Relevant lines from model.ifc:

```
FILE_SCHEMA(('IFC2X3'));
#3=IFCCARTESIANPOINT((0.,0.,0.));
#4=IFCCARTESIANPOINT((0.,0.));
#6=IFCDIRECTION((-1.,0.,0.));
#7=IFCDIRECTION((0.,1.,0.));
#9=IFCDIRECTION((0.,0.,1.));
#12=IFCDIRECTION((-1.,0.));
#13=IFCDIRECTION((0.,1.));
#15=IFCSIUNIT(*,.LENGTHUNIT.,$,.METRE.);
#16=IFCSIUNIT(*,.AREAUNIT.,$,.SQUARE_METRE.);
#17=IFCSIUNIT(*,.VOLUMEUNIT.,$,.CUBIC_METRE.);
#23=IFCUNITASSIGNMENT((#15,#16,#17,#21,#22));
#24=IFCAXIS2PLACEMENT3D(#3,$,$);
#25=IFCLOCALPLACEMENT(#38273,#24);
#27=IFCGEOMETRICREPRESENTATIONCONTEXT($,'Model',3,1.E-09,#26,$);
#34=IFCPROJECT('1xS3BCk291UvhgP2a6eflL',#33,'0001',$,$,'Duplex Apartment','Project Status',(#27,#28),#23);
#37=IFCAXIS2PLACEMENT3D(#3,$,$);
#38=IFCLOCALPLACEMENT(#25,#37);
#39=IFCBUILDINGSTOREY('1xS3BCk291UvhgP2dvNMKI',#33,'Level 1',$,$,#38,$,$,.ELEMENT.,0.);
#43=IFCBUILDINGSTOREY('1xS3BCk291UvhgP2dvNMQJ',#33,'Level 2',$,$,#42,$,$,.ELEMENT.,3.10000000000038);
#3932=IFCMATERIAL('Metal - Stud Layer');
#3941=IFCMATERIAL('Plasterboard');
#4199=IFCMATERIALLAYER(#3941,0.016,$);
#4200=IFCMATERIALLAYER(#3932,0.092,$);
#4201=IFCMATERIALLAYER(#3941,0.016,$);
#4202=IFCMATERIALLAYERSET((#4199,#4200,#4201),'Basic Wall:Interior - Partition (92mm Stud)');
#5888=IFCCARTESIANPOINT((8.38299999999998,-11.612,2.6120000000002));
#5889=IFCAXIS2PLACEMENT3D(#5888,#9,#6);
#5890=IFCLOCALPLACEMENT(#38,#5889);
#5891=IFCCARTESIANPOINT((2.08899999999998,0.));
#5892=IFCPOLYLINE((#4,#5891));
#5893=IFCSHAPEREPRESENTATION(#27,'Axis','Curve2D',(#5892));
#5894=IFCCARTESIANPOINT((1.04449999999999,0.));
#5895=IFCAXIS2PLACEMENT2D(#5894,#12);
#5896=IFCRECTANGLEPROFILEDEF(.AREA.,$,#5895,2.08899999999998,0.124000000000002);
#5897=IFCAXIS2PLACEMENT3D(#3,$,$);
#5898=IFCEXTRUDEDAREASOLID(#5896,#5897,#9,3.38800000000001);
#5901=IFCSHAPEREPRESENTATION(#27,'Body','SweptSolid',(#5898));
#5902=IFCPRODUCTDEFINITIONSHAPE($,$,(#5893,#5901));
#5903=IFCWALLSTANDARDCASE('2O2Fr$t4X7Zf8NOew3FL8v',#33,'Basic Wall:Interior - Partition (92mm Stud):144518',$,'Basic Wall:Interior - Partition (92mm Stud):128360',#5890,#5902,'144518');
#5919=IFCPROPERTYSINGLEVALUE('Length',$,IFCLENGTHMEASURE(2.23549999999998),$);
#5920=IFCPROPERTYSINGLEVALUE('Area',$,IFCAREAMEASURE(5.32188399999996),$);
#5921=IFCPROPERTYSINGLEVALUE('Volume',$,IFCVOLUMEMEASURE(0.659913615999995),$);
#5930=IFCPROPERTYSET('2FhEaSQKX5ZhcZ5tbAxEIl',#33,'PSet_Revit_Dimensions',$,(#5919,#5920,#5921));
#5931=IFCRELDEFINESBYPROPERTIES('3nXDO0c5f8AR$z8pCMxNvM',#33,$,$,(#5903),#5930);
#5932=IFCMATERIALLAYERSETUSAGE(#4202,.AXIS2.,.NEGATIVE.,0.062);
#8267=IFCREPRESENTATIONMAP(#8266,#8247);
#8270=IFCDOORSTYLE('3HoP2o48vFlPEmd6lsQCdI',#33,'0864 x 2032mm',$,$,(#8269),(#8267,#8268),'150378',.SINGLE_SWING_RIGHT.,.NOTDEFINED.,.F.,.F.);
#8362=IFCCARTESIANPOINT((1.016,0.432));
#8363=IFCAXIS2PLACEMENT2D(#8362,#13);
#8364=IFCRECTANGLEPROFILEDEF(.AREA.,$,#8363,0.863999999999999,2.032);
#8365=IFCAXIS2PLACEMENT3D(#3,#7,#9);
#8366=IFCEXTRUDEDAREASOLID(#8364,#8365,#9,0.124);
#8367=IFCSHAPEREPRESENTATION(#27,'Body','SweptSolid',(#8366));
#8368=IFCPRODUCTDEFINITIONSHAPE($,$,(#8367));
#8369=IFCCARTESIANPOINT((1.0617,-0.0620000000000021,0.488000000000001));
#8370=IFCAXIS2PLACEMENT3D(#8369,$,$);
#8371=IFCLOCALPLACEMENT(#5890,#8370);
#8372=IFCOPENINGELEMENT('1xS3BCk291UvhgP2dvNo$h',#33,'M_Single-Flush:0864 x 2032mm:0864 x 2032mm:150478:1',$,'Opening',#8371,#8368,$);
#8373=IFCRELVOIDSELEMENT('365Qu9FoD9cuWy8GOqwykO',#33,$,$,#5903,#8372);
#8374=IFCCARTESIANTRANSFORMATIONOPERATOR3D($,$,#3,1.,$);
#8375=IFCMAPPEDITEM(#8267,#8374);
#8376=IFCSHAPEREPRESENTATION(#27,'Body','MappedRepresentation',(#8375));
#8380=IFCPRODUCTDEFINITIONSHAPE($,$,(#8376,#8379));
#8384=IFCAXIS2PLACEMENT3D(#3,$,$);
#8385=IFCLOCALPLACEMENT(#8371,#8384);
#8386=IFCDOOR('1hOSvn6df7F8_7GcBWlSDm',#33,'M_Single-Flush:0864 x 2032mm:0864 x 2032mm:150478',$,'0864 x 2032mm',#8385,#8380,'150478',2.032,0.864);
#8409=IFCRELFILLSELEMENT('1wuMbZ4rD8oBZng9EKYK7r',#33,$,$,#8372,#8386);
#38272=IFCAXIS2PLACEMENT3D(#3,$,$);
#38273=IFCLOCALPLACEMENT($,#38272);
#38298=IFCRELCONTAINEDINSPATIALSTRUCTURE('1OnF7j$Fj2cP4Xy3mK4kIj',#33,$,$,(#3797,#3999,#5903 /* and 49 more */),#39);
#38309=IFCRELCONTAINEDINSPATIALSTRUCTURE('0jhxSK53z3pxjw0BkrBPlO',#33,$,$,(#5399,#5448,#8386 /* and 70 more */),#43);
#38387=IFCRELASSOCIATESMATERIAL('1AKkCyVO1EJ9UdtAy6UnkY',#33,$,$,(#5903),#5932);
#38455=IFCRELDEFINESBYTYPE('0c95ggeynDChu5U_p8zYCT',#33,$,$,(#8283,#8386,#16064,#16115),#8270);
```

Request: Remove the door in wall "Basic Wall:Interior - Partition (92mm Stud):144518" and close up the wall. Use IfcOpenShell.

```python
import ifcopenshell
import ifcopenshell.api.feature
import ifcopenshell.api.pset
import ifcopenshell.api.root
import ifcopenshell.geom
import ifcopenshell.util.element
import ifcopenshell.util.shape
import ifcopenshell.util.unit

model = ifcopenshell.open("model.ifc")
area_scale = ifcopenshell.util.unit.calculate_unit_scale(model, "AREAUNIT")
volume_scale = ifcopenshell.util.unit.calculate_unit_scale(model, "VOLUMEUNIT")
settings = ifcopenshell.geom.settings()


def volume(element):
    """Net volume in cubic metres, openings subtracted."""
    shape = ifcopenshell.geom.create_shape(settings, element)
    return ifcopenshell.util.shape.get_volume(shape.geometry)


door = model.by_guid("1hOSvn6df7F8_7GcBWlSDm")
opening = door.FillsVoids[0].RelatingOpeningElement
wall = opening.VoidsElements[0].RelatingBuildingElement
before = volume(wall)

ifcopenshell.api.root.remove_product(model, product=door)
ifcopenshell.api.feature.remove_feature(model, feature=opening)

after = volume(wall)
thickness = 0.124  # wall thickness in metres

# Update the wall's stored quantities.
pset = model.by_id(ifcopenshell.util.element.get_pset(wall, "PSet_Revit_Dimensions", should_inherit=False)["id"])
ifcopenshell.api.pset.edit_pset(model, pset=pset, properties={
    "Area": model.create_entity("IfcAreaMeasure", after / thickness / area_scale),
    "Volume": model.create_entity("IfcVolumeMeasure", after / volume_scale),
})

print(f"wall volume {before:.3f} -> {after:.3f} m3")

model.write("model_rev.ifc")
```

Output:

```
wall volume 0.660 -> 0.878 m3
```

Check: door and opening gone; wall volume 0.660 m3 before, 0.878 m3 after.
